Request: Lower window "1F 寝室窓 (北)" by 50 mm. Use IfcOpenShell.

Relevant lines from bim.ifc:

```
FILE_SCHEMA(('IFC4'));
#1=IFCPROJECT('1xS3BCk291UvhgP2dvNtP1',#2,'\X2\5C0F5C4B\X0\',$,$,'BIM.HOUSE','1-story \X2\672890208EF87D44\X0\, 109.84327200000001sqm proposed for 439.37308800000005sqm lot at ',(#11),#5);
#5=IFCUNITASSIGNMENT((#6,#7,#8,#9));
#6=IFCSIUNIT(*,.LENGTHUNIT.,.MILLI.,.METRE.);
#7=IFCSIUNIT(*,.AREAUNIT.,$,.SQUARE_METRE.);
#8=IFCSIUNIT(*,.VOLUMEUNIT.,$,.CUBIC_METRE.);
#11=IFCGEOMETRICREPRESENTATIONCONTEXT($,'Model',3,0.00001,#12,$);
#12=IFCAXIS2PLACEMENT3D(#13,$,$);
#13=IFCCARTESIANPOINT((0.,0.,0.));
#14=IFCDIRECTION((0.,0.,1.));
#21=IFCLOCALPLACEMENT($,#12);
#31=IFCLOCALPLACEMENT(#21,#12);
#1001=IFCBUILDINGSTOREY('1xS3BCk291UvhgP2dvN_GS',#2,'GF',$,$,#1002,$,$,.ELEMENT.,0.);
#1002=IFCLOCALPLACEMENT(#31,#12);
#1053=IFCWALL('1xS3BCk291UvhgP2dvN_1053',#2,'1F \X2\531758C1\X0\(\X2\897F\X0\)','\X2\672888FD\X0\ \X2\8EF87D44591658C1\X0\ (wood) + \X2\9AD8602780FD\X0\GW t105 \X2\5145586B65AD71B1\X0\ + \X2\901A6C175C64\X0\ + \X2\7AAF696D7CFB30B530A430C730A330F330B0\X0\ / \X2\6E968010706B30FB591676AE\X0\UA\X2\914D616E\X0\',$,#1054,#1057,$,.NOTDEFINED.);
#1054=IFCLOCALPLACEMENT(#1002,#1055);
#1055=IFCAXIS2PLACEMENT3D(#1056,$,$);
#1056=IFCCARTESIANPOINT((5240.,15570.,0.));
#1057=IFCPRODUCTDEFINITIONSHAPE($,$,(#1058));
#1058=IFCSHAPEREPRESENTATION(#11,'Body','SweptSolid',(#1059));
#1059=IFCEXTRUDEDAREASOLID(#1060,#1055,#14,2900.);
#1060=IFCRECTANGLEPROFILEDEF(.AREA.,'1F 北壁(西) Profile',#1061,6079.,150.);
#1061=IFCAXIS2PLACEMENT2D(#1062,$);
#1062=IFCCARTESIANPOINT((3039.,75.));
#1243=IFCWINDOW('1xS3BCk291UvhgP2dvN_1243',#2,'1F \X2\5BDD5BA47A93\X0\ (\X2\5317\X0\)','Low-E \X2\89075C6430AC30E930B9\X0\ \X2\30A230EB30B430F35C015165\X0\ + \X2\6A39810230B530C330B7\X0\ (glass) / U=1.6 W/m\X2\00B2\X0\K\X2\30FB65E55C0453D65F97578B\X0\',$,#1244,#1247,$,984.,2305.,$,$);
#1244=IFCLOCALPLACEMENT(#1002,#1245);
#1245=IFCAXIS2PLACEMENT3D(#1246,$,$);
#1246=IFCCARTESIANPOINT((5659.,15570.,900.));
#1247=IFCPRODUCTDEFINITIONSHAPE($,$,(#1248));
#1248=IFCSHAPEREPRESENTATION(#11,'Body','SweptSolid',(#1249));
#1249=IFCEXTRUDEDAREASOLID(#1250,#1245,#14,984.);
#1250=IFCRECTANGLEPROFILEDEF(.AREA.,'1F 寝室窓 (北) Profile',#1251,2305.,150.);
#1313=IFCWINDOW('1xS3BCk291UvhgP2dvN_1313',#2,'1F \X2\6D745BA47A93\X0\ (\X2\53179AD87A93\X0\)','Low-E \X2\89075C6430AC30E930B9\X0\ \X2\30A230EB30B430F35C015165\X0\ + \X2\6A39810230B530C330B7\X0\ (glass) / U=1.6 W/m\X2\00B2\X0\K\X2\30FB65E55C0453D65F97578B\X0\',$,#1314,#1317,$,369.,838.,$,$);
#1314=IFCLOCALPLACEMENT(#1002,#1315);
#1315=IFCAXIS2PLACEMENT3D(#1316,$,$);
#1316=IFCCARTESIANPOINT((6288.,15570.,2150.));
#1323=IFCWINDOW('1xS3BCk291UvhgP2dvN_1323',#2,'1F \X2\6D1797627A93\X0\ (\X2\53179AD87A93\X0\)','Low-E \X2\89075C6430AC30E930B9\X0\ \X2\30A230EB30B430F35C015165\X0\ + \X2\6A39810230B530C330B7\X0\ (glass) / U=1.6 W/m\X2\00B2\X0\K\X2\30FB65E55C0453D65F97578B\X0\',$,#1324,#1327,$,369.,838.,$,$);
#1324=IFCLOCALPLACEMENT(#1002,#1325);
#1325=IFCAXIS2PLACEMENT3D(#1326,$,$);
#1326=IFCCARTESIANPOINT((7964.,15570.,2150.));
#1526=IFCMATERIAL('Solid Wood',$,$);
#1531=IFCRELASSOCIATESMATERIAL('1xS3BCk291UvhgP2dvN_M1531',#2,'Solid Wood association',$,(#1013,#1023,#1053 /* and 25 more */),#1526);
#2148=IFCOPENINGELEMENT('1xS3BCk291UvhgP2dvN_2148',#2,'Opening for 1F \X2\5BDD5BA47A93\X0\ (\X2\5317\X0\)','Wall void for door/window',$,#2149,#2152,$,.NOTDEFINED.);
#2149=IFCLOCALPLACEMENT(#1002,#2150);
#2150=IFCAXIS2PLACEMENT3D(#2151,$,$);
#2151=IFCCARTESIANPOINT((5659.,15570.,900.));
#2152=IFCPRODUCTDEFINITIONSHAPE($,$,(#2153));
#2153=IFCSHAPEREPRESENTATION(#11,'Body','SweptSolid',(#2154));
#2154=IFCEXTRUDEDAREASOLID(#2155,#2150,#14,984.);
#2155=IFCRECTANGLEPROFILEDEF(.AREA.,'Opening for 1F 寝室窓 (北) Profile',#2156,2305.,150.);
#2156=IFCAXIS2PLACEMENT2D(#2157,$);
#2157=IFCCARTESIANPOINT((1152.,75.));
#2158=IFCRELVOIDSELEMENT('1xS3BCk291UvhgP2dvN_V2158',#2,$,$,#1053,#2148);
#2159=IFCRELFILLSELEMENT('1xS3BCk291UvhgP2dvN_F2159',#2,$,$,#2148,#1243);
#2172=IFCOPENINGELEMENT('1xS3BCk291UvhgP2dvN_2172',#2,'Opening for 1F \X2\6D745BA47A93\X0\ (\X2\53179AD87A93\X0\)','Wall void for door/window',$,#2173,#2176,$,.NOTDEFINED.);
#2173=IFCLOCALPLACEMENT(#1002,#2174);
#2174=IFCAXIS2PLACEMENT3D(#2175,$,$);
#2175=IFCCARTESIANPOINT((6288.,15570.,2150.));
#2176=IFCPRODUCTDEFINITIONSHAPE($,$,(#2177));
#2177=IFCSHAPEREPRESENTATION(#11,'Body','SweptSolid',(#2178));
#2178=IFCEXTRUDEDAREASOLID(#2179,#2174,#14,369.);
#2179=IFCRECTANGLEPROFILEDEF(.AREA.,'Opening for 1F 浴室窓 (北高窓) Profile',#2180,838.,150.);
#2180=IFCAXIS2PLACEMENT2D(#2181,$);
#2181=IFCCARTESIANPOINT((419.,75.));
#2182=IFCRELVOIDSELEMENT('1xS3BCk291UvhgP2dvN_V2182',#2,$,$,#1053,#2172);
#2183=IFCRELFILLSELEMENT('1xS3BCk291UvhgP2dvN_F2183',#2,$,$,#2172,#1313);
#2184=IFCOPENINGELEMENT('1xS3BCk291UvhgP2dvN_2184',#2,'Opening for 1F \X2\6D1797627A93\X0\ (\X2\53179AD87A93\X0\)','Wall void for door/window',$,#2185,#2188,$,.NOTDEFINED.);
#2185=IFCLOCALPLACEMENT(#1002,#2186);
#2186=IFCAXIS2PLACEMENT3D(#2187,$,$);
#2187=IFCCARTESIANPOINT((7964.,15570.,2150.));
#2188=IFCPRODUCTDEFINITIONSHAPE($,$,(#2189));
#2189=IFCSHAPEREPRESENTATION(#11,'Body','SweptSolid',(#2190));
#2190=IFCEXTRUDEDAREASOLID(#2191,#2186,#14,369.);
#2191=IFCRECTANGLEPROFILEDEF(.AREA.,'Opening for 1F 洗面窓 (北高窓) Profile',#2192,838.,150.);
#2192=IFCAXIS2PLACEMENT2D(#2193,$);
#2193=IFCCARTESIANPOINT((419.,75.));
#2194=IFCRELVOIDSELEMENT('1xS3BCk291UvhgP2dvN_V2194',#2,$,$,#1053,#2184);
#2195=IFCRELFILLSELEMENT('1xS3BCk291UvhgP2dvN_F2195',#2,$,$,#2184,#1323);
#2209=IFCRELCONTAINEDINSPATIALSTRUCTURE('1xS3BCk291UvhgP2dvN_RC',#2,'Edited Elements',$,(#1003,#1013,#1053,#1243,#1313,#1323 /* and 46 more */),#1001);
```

```python
import numpy as np
import ifcopenshell
import ifcopenshell.api.geometry
import ifcopenshell.util.placement
import ifcopenshell.util.unit

model = ifcopenshell.open("bim.ifc")
unit_scale = ifcopenshell.util.unit.calculate_unit_scale(model)

window = model.by_guid("1xS3BCk291UvhgP2dvN_1243")
opening = window.FillsVoids[0].RelatingOpeningElement
dz = -0.05 / unit_scale

shift = np.array([0.0, 0.0, dz])
# The window is not placed relative to its opening, so move both.
for product in (opening, window):
    matrix = ifcopenshell.util.placement.get_local_placement(product.ObjectPlacement)
    matrix[:3, 3] += shift
    ifcopenshell.api.geometry.edit_object_placement(model, product=product, matrix=matrix, is_si=False)

print(f"moved by {dz * unit_scale:+.3f} m")

model.write("bim_edited.ifc")
```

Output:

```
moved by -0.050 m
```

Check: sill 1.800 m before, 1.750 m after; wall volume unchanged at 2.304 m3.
